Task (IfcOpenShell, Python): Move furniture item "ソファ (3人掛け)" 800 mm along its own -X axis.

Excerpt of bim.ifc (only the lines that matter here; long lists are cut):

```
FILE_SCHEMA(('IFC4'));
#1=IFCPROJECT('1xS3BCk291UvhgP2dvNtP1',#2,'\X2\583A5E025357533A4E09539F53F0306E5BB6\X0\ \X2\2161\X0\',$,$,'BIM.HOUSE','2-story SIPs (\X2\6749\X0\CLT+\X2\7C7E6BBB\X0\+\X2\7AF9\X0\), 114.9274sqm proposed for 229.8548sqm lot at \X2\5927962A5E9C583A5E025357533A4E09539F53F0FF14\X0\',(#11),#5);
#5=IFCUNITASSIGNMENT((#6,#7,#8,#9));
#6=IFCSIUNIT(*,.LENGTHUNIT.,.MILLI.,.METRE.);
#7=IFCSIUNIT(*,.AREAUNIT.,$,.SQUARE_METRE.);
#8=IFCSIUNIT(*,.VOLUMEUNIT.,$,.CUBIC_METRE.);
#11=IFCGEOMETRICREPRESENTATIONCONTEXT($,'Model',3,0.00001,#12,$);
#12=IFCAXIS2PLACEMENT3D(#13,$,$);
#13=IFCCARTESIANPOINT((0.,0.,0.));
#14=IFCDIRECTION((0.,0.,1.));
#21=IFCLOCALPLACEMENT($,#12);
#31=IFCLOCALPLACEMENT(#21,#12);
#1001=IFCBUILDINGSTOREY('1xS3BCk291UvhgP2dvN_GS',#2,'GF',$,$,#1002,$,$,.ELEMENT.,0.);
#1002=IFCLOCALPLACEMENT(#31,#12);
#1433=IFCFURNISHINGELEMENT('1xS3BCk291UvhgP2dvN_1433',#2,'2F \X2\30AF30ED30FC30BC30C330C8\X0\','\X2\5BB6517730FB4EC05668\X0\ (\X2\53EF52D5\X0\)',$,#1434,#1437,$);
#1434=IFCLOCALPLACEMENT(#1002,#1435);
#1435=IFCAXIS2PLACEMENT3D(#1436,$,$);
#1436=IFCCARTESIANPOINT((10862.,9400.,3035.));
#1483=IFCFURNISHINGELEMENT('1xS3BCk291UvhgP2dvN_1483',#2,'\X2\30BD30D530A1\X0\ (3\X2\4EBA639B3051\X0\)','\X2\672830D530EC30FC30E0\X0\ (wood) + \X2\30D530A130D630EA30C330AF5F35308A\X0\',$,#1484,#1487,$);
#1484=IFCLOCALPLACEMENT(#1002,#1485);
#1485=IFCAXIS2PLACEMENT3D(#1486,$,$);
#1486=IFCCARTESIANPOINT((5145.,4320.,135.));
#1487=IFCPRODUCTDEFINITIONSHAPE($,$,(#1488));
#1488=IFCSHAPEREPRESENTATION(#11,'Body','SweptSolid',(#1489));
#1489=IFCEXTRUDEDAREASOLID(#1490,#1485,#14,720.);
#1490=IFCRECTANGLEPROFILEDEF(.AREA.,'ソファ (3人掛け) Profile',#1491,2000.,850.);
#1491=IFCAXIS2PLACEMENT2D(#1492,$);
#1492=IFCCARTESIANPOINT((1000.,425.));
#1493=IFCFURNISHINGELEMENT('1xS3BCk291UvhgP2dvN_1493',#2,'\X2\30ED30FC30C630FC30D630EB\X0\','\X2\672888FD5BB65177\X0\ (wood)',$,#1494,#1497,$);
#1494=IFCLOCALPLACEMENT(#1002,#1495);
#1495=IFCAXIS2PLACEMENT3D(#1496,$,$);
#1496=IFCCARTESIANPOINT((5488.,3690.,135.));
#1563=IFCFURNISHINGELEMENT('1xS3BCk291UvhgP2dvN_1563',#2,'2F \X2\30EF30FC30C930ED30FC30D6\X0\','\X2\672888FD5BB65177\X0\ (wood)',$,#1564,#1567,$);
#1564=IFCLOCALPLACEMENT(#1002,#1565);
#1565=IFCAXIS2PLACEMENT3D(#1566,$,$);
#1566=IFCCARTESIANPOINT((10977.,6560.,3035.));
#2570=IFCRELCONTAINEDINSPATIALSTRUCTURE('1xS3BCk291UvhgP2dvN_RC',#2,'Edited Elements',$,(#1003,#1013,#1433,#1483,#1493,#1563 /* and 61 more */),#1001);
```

```python
import ifcopenshell
import ifcopenshell.api.geometry
import ifcopenshell.util.placement

model = ifcopenshell.open("bim.ifc")

item = model.by_guid("1xS3BCk291UvhgP2dvN_1483")
matrix = ifcopenshell.util.placement.get_local_placement(item.ObjectPlacement)
matrix[:3, 3] -= matrix[:3, 0] * 800.0
ifcopenshell.api.geometry.edit_object_placement(model, product=item, matrix=matrix, is_si=False)

print(ifcopenshell.util.placement.get_local_placement(item.ObjectPlacement).round(3) + 0.0)

model.write("bim_edited.ifc")
```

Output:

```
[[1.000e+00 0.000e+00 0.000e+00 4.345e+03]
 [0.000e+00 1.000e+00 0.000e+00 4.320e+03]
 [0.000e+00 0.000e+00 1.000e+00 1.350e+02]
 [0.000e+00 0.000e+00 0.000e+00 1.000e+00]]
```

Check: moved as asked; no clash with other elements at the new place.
